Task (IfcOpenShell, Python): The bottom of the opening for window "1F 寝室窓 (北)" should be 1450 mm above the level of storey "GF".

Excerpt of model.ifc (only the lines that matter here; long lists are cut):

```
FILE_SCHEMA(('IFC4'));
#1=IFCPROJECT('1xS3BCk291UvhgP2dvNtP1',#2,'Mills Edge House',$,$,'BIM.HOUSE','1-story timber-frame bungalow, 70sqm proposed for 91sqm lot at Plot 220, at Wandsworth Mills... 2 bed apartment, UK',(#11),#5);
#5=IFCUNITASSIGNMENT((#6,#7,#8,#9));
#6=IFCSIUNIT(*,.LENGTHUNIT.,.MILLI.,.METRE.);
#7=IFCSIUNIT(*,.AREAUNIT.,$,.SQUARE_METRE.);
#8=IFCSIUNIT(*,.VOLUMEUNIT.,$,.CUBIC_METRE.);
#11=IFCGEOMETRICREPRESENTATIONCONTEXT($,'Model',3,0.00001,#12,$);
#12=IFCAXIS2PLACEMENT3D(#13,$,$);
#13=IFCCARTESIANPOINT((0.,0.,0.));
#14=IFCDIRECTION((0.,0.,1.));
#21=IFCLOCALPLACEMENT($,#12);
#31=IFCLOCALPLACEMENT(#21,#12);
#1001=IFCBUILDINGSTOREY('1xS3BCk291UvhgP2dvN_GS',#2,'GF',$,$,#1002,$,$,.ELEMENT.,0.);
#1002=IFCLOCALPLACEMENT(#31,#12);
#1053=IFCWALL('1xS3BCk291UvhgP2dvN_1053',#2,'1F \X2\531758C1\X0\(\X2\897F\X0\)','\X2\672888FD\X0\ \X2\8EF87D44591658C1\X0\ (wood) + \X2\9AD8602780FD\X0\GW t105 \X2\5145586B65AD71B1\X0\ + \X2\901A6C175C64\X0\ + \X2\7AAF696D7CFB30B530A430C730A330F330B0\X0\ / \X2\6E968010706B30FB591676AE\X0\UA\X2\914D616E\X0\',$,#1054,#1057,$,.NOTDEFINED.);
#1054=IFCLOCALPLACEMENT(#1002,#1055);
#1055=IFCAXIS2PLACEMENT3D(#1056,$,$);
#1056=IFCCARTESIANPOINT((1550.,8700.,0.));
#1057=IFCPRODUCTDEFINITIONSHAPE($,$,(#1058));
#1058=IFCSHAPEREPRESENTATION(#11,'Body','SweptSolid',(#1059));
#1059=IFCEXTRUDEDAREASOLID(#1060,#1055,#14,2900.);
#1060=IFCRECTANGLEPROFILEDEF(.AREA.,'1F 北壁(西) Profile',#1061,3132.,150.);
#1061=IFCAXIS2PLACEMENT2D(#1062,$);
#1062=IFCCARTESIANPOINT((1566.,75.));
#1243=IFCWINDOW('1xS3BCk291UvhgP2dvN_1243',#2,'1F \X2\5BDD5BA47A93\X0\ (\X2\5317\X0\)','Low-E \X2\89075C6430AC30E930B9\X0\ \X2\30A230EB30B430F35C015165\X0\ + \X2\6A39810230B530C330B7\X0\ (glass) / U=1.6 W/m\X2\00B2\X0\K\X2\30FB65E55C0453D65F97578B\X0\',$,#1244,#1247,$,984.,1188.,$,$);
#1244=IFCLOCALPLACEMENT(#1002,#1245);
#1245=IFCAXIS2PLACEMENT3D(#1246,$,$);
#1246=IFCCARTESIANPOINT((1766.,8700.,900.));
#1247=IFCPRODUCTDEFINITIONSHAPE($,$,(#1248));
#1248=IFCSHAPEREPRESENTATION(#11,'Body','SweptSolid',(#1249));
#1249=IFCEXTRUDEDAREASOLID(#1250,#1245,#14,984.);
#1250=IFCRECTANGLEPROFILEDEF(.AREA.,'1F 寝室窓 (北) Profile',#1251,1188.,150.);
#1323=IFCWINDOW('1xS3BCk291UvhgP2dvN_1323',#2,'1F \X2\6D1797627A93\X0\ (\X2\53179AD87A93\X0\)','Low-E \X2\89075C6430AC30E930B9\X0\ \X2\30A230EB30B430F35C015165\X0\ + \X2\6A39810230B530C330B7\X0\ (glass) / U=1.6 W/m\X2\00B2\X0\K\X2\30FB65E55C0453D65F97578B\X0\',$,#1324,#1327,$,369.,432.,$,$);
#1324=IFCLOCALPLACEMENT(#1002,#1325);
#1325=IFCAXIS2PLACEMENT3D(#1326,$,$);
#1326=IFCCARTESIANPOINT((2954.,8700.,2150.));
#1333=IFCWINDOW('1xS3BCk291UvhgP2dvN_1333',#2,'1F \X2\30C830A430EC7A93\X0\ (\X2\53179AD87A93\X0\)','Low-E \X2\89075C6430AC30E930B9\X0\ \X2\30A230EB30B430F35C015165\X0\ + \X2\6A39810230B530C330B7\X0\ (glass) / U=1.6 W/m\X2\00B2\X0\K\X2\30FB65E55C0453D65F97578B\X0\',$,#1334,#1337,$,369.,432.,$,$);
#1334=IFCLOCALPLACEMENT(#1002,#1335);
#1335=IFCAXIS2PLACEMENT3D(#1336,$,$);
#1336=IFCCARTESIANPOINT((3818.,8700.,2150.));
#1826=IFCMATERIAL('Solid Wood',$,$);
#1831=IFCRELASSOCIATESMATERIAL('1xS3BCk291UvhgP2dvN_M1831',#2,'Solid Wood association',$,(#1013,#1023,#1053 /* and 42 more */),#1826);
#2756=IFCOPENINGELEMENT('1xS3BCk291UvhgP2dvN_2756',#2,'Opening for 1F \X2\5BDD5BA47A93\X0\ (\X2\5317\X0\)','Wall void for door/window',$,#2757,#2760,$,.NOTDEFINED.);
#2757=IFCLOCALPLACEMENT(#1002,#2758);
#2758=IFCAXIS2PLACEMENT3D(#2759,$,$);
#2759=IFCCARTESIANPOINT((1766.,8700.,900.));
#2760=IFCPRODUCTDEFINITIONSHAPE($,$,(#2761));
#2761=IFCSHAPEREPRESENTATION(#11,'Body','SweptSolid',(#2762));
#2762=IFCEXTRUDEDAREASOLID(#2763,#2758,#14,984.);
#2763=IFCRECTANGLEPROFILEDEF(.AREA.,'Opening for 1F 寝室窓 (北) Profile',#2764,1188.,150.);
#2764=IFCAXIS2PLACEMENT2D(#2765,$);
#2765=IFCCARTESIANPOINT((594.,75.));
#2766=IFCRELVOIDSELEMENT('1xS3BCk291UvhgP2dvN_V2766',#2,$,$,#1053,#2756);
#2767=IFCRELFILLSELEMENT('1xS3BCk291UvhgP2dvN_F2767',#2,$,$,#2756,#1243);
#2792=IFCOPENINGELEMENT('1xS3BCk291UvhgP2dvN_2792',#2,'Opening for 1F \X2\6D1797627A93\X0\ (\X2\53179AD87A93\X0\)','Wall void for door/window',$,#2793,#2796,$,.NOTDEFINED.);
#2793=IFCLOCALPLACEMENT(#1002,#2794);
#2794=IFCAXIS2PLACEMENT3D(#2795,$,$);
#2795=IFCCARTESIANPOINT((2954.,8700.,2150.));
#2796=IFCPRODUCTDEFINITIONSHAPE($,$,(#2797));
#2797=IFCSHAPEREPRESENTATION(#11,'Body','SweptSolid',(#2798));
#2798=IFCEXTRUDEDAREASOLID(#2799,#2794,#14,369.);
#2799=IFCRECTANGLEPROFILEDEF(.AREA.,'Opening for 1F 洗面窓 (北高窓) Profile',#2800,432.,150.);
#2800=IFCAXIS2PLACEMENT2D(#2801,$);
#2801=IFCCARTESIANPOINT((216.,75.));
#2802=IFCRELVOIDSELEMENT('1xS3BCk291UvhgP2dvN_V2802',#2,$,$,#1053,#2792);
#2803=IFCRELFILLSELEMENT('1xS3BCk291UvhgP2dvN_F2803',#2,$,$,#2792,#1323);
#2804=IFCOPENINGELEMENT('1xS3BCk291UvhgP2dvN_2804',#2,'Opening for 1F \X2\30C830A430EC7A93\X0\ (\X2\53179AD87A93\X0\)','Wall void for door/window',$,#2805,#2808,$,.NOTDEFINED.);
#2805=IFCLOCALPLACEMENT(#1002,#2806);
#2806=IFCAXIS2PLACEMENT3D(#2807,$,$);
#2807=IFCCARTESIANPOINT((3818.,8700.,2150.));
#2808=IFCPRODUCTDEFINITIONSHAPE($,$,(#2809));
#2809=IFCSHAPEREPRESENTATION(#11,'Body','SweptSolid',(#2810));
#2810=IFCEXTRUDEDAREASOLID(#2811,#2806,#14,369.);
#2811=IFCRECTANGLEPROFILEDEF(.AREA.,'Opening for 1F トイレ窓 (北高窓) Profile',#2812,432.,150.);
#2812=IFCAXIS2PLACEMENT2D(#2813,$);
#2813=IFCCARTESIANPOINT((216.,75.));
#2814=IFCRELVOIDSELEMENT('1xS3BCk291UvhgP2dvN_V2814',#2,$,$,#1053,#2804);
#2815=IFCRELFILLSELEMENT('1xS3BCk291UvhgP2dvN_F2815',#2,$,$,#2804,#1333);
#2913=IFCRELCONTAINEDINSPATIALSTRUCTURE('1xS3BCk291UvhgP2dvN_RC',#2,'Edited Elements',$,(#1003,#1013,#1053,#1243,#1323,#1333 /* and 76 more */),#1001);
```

```python
import numpy as np
import ifcopenshell
import ifcopenshell.api.geometry
import ifcopenshell.geom
import ifcopenshell.util.element
import ifcopenshell.util.placement
import ifcopenshell.util.shape
import ifcopenshell.util.unit

model = ifcopenshell.open("model.ifc")
unit_scale = ifcopenshell.util.unit.calculate_unit_scale(model)

window = model.by_id(1243)
opening = window.FillsVoids[0].RelatingOpeningElement
storey = ifcopenshell.util.element.get_container(window, ifc_class="IfcBuildingStorey")
level = ifcopenshell.util.placement.get_local_placement(storey.ObjectPlacement)[2, 3]

# The opening's origin need not be at the sill, so measure its lowest point.
shape = ifcopenshell.geom.create_shape(ifcopenshell.geom.settings(), opening)
bottom = ifcopenshell.util.shape.get_shape_bottom_elevation(shape, shape.geometry) / unit_scale
dz = level + 1450.0 - bottom

shift = np.array([0.0, 0.0, dz])
# The window is not placed relative to its opening, so move both.
for product in (opening, window):
    matrix = ifcopenshell.util.placement.get_local_placement(product.ObjectPlacement)
    matrix[:3, 3] += shift
    ifcopenshell.api.geometry.edit_object_placement(model, product=product, matrix=matrix, is_si=False)

print(f"moved by {dz * unit_scale:+.3f} m")

model.write("model_v2.ifc")
```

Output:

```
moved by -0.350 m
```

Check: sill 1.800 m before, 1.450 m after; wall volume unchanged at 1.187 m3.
